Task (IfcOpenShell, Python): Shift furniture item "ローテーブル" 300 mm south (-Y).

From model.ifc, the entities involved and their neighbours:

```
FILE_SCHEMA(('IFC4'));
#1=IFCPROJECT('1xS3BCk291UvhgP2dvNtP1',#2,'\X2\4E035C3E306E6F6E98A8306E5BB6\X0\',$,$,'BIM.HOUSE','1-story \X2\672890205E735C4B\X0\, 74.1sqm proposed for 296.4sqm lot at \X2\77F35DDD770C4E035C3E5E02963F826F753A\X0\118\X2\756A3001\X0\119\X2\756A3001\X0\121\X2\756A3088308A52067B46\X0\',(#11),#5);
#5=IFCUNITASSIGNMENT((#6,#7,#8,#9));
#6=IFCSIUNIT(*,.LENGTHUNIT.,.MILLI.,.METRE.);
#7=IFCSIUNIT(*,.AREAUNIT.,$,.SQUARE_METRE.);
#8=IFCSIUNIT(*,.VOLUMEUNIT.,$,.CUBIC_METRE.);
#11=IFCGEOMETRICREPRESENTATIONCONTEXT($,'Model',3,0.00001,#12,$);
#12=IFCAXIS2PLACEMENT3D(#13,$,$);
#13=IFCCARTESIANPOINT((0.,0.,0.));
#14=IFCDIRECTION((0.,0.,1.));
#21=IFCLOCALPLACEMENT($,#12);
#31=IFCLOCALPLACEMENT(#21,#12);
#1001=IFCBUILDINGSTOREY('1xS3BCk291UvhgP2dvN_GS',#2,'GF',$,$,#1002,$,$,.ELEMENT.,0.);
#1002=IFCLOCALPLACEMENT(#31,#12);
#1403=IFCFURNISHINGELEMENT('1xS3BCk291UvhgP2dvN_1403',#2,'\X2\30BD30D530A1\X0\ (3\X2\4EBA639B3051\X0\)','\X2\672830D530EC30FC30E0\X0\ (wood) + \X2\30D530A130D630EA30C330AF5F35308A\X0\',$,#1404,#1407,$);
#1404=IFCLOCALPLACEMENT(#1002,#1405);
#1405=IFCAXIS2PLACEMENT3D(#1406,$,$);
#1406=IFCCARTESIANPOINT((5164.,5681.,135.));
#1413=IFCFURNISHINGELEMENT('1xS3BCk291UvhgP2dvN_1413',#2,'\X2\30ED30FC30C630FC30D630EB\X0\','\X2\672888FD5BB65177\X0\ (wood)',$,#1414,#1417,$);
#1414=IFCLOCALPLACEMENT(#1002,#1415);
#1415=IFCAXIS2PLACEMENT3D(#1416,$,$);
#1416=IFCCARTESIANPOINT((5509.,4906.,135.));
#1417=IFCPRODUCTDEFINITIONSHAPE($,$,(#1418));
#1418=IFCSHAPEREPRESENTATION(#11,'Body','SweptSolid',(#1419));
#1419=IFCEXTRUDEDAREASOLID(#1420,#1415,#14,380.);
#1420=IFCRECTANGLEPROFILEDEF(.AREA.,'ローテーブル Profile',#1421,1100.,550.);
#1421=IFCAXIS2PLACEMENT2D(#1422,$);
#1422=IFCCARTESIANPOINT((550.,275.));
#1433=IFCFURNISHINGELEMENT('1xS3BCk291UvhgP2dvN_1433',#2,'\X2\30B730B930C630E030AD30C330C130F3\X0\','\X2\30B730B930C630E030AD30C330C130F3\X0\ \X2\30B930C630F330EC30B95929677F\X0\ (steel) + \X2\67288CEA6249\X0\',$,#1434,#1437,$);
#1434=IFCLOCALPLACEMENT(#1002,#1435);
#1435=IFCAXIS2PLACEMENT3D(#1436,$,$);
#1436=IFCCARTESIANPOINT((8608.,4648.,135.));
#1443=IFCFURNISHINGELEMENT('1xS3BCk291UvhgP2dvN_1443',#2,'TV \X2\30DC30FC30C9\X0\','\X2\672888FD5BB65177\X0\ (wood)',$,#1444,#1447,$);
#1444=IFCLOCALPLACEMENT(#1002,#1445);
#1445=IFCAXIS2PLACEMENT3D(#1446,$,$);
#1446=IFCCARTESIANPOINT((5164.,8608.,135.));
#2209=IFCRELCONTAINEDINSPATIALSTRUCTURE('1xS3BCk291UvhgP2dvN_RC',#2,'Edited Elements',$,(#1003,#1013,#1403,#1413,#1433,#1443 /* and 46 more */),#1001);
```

```python
import ifcopenshell
import ifcopenshell.api.geometry
import ifcopenshell.util.placement
import ifcopenshell.util.unit

model = ifcopenshell.open("model.ifc")
unit_scale = ifcopenshell.util.unit.calculate_unit_scale(model)

item = model.by_guid("1xS3BCk291UvhgP2dvN_1413")
matrix = ifcopenshell.util.placement.get_local_placement(item.ObjectPlacement)
matrix[1, 3] -= 0.3 / unit_scale
ifcopenshell.api.geometry.edit_object_placement(model, product=item, matrix=matrix, is_si=False)

print(ifcopenshell.util.placement.get_local_placement(item.ObjectPlacement).round(3) + 0.0)

model.write("model_edited.ifc")
```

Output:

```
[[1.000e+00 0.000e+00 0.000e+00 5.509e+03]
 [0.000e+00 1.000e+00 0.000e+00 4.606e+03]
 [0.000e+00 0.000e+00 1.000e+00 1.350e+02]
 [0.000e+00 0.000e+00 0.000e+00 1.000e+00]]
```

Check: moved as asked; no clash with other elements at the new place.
